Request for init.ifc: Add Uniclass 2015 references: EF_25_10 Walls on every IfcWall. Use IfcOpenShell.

First a look at what the model holds.

```python
import ifcopenshell

model = ifcopenshell.open("init.ifc")
print(model.schema)
print("classifications:", [c.Name for c in model.by_type("IfcClassification")])
for ifc_class in ("IfcDoor", "IfcRoof", "IfcStair", "IfcWall", "IfcWindow"):
    print(ifc_class, len(model.by_type(ifc_class)))
```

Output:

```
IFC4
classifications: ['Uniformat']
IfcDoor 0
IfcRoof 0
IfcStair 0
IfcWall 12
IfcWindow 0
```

```python
import ifcopenshell
import ifcopenshell.api.classification

model = ifcopenshell.open("init.ifc")

system = ifcopenshell.api.classification.add_classification(model, classification="Uniclass 2015")

codes = {
    "IfcWall": ("EF_25_10", "Walls"),
}
for ifc_class, (code, name) in codes.items():
    products = model.by_type(ifc_class)
    ifcopenshell.api.classification.add_reference(
        model, products=products, classification=system, identification=code, name=name
    )
    print(code, len(products))

model.write("init_rev.ifc")
```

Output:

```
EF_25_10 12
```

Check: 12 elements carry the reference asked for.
